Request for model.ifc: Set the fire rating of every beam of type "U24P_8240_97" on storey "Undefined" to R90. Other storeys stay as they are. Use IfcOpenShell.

First a look at what the model holds.

```python
import ifcopenshell
import ifcopenshell.util.element

model = ifcopenshell.open("model.ifc")
print(model.schema)
storey = next(s for s in model.by_type("IfcBuildingStorey") if s.Name == "Undefined")
beams = [e for e in ifcopenshell.util.element.get_decomposition(storey) if e.is_a("IfcBeam")]
seen = {}
for e in beams:
    element_type = ifcopenshell.util.element.get_type(e)
    key = (element_type.Name if element_type != e and element_type else None, ifcopenshell.util.element.get_pset(e, "Pset_BeamCommon", "FireRating"))
    seen[key] = seen.get(key, 0) + 1
for (name, value), count in sorted(seen.items(), key=str):
    print(count, "x", name, "|", value)
```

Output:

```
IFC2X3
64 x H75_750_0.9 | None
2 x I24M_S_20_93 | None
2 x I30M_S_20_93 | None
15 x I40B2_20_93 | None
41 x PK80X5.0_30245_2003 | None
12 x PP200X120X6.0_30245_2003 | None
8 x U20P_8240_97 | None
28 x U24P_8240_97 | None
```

```python
import ifcopenshell
import ifcopenshell.api.pset
import ifcopenshell.util.element

model = ifcopenshell.open("model.ifc")

storey = next(s for s in model.by_type("IfcBuildingStorey") if s.Name == "Undefined")
beams = [e for e in ifcopenshell.util.element.get_decomposition(storey) if e.is_a("IfcBeam")]

count = 0
for e in beams:
    element_type = ifcopenshell.util.element.get_type(e)
    if element_type in (None, e) or element_type.Name != "U24P_8240_97":
        continue
    found = ifcopenshell.util.element.get_pset(e, "Pset_BeamCommon", should_inherit=False)
    if found:
        pset = model.by_id(found["id"])
        if len(ifcopenshell.util.element.get_elements_by_pset(pset)) > 1:
            pset = ifcopenshell.api.pset.unshare_pset(model, products=[e], pset=pset)[0]
    else:
        pset = ifcopenshell.api.pset.add_pset(model, product=e, name="Pset_BeamCommon")
    ifcopenshell.api.pset.edit_pset(model, pset=pset, properties={"FireRating": "R90"})
    count += 1

print(count, "beams updated")

model.write("model_rev.ifc")
```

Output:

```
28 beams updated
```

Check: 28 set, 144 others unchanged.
